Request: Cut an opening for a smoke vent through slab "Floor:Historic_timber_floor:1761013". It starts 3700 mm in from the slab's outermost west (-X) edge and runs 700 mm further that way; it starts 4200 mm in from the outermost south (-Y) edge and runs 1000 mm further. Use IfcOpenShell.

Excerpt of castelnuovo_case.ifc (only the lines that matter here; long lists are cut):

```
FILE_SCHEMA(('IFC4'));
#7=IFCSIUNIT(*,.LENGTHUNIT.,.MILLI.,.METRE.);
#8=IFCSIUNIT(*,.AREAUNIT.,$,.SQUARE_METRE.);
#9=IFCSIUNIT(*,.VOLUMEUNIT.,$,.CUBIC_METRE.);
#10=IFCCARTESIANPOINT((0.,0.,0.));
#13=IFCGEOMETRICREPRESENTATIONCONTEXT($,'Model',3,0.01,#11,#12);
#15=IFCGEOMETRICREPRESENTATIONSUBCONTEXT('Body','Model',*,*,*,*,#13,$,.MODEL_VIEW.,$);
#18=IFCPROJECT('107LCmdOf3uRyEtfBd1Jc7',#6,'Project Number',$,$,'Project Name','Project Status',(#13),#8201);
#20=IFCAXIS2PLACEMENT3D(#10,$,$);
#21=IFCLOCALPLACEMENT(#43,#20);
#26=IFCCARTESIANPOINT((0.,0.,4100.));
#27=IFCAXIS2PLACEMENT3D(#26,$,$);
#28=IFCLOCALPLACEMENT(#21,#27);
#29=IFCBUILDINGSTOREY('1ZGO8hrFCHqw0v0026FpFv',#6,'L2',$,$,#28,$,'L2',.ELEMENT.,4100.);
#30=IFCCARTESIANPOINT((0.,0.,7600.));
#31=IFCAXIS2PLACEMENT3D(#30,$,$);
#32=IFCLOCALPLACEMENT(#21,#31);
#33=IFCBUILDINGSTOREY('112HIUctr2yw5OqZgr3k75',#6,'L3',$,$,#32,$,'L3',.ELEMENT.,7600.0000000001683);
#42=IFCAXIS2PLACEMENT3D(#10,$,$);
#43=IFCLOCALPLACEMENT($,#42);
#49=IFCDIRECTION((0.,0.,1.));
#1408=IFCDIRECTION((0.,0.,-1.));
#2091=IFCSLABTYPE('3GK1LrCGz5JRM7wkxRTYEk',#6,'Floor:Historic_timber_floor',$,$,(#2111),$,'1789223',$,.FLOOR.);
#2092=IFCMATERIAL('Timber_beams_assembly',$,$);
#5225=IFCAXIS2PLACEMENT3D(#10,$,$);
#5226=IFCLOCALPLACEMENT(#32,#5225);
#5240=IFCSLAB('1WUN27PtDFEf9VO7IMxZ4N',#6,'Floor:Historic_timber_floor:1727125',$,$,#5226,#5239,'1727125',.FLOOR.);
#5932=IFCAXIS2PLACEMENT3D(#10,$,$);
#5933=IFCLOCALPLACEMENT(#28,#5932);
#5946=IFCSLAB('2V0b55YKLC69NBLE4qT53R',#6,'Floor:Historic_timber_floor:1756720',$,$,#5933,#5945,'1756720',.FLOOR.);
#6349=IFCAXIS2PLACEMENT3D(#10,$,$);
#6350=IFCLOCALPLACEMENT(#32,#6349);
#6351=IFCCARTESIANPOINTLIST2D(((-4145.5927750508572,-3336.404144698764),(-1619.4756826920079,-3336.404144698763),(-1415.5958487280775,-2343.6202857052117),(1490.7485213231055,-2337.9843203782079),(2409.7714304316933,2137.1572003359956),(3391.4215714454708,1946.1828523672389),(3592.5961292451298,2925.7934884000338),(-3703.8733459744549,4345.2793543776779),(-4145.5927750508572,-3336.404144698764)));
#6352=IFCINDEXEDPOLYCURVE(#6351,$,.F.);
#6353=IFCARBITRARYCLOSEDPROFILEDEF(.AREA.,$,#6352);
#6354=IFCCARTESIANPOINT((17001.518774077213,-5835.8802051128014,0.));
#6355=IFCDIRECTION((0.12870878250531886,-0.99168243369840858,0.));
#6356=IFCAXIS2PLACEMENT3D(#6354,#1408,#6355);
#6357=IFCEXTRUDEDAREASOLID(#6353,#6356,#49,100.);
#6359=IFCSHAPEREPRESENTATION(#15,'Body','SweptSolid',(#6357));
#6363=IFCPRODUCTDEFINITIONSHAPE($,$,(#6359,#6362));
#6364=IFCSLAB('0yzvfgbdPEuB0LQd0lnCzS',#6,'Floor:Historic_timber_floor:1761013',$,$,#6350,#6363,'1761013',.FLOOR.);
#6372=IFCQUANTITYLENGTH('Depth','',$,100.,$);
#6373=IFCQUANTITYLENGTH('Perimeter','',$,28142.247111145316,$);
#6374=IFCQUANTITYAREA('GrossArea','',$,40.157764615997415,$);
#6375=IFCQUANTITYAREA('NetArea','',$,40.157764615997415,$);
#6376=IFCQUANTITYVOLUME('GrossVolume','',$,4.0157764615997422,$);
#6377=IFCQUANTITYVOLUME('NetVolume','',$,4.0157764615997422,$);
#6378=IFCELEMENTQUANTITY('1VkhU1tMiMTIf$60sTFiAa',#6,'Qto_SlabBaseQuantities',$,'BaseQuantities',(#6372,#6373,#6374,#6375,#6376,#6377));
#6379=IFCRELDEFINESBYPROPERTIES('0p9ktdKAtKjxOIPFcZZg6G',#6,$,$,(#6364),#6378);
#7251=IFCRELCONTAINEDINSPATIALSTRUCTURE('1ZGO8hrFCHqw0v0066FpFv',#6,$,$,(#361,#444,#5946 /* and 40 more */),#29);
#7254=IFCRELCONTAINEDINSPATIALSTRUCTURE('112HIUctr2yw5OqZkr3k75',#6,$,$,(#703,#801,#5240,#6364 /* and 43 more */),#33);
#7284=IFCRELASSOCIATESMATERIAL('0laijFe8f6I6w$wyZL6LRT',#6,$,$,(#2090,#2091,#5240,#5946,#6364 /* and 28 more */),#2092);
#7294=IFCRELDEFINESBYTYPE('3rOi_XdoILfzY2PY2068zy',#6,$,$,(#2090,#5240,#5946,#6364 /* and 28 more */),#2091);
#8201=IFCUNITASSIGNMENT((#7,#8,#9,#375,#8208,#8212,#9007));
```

```python
import numpy as np
import ifcopenshell
import ifcopenshell.api.feature
import ifcopenshell.api.geometry
import ifcopenshell.api.pset
import ifcopenshell.api.root
import ifcopenshell.geom
import ifcopenshell.util.element
import ifcopenshell.util.placement
import ifcopenshell.util.representation
import ifcopenshell.util.shape
import ifcopenshell.util.unit

model = ifcopenshell.open("castelnuovo_case.ifc")
unit_scale = ifcopenshell.util.unit.calculate_unit_scale(model)
area_scale = ifcopenshell.util.unit.calculate_unit_scale(model, "AREAUNIT")
volume_scale = ifcopenshell.util.unit.calculate_unit_scale(model, "VOLUMEUNIT")
settings = ifcopenshell.geom.settings()


def volume(element):
    """Net volume in cubic metres, openings subtracted."""
    shape = ifcopenshell.geom.create_shape(settings, element)
    return ifcopenshell.util.shape.get_volume(shape.geometry)


slab = model.by_guid("0yzvfgbdPEuB0LQd0lnCzS")
before = volume(slab)

# Extent in the slab's own axes, in metres. The edges named are its -X and -Y sides.
slab_shape = ifcopenshell.geom.create_shape(settings, slab)
vertices = ifcopenshell.util.shape.get_vertices(slab_shape.geometry)
x_min, y_min, bottom = vertices.min(axis=0)
top = vertices[:, 2].max()

opening = ifcopenshell.api.root.create_entity(model, ifc_class="IfcOpeningElement", name="Smoke vent opening", predefined_type="OPENING")
context = ifcopenshell.util.representation.get_context(model, "Model", "Body", "MODEL_VIEW")
width, depth = 0.7, 1
outline = [(0.0, 0.0), (width, 0.0), (width, depth), (0.0, depth), (0.0, 0.0)]
# Overshoot both faces by 50 mm so the cut is clean.
shape = ifcopenshell.api.geometry.add_slab_representation(
    model, context=context, depth=top - bottom + 0.1, polyline=outline
)
ifcopenshell.api.geometry.assign_representation(model, product=opening, representation=shape)

matrix = ifcopenshell.util.placement.get_local_placement(slab.ObjectPlacement)
matrix[:, 3] = matrix @ np.append(np.array([x_min + 3.7, y_min + 4.2, bottom - 0.05]) / unit_scale, 1.0)
ifcopenshell.api.geometry.edit_object_placement(model, product=opening, matrix=matrix, is_si=False)
ifcopenshell.api.feature.add_feature(model, feature=opening, element=slab)

after = volume(slab)

# Update the slab's stored quantities.
qto = model.by_id(ifcopenshell.util.element.get_pset(slab, "Qto_SlabBaseQuantities", should_inherit=False)["id"])
ifcopenshell.api.pset.edit_qto(model, qto=qto, properties={
    "NetArea": after / (top - bottom) / area_scale,
    "NetVolume": after / volume_scale,
})

print(f"slab volume {before:.3f} -> {after:.3f} m3")

model.write("castelnuovo_case_updated.ifc")
```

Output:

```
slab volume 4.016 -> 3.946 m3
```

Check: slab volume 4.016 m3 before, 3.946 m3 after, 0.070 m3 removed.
